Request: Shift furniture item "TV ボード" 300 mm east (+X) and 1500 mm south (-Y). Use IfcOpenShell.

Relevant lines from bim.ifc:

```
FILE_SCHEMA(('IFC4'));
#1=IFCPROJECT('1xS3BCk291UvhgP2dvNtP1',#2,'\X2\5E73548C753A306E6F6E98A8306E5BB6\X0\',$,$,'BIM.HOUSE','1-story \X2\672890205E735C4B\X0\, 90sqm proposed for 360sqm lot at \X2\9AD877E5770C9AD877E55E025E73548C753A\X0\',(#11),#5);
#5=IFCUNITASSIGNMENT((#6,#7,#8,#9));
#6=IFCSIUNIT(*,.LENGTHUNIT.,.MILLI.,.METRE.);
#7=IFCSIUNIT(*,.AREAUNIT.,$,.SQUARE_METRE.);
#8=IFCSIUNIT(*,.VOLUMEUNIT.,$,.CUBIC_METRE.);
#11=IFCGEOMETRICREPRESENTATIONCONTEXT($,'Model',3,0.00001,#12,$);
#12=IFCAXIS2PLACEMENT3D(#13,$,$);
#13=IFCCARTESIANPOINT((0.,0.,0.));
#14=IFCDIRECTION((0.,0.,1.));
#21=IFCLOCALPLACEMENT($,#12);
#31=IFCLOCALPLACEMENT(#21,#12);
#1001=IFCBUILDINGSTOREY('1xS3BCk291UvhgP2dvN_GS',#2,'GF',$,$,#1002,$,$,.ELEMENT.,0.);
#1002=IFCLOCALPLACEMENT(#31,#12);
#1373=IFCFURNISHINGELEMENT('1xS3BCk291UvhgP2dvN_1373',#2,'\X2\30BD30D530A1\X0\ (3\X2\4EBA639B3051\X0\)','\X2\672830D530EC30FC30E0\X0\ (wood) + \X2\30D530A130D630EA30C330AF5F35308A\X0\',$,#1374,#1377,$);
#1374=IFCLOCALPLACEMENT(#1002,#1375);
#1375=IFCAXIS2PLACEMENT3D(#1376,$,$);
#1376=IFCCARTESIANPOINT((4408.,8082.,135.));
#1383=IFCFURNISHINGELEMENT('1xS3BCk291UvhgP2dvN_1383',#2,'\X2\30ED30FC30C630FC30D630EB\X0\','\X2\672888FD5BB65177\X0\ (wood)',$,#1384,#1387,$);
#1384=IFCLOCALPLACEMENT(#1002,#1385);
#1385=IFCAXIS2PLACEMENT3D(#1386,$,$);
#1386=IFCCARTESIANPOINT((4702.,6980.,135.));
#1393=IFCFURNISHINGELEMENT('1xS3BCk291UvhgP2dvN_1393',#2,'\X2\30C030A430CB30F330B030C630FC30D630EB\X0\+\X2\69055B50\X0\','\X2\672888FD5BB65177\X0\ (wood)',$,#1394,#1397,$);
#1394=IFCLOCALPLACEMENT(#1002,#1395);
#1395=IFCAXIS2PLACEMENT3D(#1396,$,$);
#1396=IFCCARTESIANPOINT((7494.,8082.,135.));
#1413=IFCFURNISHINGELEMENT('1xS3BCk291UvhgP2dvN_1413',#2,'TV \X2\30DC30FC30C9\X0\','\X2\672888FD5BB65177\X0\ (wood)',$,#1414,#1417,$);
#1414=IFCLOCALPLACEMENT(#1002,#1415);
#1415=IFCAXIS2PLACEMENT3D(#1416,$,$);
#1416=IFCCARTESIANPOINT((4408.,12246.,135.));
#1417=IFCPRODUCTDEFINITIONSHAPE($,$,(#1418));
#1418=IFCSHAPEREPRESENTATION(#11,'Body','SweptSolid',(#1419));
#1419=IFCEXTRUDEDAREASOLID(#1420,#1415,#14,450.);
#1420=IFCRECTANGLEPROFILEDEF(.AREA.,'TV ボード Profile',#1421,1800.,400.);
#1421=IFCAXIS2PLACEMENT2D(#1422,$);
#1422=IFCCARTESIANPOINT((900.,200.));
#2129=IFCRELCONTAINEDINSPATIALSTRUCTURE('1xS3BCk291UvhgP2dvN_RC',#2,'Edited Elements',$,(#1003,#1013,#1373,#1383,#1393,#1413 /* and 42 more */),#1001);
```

```python
import ifcopenshell
import ifcopenshell.api.geometry
import ifcopenshell.util.placement

model = ifcopenshell.open("bim.ifc")

item = model.by_id(1413)
matrix = ifcopenshell.util.placement.get_local_placement(item.ObjectPlacement)
matrix[0, 3] += 300.0
matrix[1, 3] -= 1500.0
ifcopenshell.api.geometry.edit_object_placement(model, product=item, matrix=matrix, is_si=False)

print(ifcopenshell.util.placement.get_local_placement(item.ObjectPlacement).round(3) + 0.0)

model.write("bim_rev.ifc")
```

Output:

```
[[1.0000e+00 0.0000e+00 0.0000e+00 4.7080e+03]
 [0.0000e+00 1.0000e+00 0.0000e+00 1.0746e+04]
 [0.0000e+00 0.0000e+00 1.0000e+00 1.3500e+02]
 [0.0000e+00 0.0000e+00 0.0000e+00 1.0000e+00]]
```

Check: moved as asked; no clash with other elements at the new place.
